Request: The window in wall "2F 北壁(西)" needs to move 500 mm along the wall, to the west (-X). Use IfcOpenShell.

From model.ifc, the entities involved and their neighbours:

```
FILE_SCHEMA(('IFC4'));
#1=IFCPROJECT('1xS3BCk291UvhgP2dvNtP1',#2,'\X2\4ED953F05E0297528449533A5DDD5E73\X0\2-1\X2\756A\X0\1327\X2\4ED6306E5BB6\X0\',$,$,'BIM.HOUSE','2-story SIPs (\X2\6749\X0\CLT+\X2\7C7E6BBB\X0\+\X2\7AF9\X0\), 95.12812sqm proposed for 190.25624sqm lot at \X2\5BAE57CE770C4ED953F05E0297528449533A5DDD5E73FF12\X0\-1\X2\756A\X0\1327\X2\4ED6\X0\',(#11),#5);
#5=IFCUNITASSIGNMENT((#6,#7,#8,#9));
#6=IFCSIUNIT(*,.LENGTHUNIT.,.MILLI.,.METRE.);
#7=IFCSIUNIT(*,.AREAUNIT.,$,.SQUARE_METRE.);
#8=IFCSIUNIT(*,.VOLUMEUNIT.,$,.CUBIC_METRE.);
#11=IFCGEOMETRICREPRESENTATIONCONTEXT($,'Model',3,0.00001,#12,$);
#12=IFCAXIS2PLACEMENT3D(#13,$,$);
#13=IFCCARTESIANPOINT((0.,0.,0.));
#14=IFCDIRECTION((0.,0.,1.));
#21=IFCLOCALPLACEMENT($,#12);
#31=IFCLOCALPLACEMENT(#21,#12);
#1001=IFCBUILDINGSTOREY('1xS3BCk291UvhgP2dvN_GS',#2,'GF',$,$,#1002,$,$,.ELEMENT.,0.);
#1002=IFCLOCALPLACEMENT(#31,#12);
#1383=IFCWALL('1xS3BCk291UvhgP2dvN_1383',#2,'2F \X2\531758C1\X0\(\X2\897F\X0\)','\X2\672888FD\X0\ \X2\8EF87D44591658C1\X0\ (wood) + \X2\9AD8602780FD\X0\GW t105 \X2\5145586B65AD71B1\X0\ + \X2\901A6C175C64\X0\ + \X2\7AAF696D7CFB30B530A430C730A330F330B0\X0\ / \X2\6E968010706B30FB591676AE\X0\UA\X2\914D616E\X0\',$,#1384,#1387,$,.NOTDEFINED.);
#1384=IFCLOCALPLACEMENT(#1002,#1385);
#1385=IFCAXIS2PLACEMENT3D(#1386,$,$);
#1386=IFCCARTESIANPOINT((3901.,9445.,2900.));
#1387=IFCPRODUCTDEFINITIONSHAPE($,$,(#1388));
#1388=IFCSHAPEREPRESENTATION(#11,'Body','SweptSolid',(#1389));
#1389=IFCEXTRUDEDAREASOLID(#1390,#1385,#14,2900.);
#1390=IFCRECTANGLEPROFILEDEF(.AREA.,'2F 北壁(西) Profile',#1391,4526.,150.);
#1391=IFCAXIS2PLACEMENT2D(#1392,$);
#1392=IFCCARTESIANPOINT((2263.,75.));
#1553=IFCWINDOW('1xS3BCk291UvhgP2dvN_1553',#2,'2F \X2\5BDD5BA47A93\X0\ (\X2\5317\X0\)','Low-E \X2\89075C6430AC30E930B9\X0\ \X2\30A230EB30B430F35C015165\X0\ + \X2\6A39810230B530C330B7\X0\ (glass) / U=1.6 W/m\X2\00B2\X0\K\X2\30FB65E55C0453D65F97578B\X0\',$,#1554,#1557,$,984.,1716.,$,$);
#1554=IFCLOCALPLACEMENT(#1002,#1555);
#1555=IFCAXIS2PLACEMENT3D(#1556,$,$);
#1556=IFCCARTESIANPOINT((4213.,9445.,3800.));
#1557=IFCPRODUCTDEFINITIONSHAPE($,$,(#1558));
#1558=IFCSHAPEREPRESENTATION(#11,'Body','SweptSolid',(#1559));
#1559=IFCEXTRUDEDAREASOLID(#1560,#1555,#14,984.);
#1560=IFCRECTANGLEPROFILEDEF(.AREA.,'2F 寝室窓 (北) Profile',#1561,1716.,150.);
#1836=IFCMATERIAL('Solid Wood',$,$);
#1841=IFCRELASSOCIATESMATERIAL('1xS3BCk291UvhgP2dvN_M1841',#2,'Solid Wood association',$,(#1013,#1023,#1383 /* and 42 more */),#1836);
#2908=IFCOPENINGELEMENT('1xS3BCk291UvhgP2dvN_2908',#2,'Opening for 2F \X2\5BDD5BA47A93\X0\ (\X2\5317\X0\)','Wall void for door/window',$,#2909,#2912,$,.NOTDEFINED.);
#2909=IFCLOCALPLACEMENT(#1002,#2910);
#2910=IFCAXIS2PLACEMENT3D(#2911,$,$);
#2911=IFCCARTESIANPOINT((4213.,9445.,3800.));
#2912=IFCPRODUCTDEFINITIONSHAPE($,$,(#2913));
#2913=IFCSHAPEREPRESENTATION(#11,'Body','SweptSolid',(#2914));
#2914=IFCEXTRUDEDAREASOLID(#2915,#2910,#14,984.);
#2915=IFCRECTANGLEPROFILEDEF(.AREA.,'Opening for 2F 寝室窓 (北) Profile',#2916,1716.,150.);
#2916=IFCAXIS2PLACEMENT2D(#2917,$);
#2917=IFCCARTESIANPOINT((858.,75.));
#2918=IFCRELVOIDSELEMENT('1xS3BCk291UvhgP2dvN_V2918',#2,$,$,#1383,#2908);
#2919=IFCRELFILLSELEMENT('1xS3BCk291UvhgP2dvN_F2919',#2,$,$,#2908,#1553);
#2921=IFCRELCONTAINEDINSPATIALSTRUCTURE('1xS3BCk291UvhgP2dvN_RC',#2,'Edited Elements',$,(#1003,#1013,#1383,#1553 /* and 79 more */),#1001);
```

```python
import ifcopenshell
import ifcopenshell.api.geometry
import ifcopenshell.util.placement
import ifcopenshell.util.unit

model = ifcopenshell.open("model.ifc")
unit_scale = ifcopenshell.util.unit.calculate_unit_scale(model)

window = model.by_guid("1xS3BCk291UvhgP2dvN_1553")
opening = window.FillsVoids[0].RelatingOpeningElement
wall = opening.VoidsElements[0].RelatingBuildingElement

wall_matrix = ifcopenshell.util.placement.get_local_placement(wall.ObjectPlacement)
shift = wall_matrix[:3, 0] * -0.5 / unit_scale
before = ifcopenshell.util.placement.get_local_placement(window.ObjectPlacement)[:3, 3].copy()

# The window is not placed relative to its opening, so move both.
for product in (opening, window):
    matrix = ifcopenshell.util.placement.get_local_placement(product.ObjectPlacement)
    matrix[:3, 3] += shift
    ifcopenshell.api.geometry.edit_object_placement(model, product=product, matrix=matrix, is_si=False)

after = ifcopenshell.util.placement.get_local_placement(window.ObjectPlacement)[:3, 3]
print("window moved by", (after - before).round(3) + 0.0)

model.write("model_edited.ifc")
```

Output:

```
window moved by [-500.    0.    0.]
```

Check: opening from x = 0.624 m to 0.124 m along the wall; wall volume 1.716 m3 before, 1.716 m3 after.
